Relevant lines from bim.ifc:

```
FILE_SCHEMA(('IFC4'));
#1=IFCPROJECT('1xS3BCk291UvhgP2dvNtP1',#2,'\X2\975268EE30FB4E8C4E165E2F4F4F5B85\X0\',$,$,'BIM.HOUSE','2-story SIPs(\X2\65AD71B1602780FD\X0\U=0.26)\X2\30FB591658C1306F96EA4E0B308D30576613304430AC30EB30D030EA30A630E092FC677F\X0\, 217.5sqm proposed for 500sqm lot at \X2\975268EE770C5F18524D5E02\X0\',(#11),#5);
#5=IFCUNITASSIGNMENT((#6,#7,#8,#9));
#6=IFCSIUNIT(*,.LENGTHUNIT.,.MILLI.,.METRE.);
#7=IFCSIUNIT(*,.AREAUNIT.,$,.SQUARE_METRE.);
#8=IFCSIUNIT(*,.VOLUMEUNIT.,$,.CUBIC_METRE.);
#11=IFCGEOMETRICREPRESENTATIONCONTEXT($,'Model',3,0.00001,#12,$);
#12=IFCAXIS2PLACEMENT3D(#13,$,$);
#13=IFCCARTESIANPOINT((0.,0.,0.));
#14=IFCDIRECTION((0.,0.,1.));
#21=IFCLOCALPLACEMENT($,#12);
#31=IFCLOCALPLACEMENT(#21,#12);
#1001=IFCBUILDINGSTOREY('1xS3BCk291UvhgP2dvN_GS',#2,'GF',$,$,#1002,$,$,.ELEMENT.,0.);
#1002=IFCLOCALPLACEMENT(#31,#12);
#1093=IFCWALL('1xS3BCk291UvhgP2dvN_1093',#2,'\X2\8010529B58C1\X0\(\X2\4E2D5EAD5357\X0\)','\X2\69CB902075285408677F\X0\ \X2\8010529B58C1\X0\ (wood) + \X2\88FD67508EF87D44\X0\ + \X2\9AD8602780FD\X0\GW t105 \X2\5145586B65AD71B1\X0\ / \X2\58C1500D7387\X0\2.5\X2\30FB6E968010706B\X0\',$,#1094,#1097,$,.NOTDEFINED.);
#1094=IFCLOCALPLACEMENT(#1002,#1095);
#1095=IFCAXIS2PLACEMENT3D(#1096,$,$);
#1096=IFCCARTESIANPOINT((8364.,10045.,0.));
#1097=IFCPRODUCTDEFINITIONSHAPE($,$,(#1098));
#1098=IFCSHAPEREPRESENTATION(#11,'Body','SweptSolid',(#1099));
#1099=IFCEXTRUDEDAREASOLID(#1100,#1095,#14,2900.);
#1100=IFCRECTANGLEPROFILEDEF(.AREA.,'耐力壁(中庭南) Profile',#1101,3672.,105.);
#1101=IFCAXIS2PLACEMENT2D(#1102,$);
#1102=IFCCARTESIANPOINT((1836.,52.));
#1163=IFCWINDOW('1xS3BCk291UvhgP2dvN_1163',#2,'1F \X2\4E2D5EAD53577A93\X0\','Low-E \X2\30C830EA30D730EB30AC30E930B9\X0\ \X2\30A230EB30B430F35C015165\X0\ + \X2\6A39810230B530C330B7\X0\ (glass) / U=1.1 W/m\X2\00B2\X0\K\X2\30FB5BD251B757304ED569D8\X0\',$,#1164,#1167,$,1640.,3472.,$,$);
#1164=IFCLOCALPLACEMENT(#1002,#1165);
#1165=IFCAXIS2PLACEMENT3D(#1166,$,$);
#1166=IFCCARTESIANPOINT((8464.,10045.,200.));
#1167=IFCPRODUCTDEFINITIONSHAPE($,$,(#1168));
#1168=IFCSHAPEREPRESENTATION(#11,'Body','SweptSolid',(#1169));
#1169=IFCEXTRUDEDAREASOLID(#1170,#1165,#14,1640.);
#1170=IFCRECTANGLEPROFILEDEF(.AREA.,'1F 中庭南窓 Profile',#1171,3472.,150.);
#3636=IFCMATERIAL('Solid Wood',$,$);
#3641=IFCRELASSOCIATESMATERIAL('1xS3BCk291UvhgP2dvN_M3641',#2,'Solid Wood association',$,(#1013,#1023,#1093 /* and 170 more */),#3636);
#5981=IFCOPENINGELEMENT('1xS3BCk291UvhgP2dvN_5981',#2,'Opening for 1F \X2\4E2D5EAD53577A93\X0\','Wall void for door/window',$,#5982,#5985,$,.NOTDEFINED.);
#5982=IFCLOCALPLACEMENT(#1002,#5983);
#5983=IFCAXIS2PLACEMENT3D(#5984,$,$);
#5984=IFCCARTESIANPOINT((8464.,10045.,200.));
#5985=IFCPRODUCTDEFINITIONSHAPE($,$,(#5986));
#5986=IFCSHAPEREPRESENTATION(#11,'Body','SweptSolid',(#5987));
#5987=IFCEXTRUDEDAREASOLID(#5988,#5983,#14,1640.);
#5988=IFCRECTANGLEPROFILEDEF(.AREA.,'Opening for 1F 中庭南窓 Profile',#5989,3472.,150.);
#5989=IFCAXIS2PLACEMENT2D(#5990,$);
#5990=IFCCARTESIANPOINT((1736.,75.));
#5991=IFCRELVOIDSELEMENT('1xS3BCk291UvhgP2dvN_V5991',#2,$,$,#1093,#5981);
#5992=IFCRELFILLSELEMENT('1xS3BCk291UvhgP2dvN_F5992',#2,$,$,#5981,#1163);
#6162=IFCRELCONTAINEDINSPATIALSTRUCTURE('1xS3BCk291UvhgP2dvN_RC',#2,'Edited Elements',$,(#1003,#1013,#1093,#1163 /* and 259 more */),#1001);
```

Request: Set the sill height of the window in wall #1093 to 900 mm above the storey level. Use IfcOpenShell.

```python
import numpy as np
import ifcopenshell
import ifcopenshell.api.geometry
import ifcopenshell.geom
import ifcopenshell.util.element
import ifcopenshell.util.placement
import ifcopenshell.util.shape
import ifcopenshell.util.unit

model = ifcopenshell.open("bim.ifc")
unit_scale = ifcopenshell.util.unit.calculate_unit_scale(model)

window = model.by_id(1163)
opening = window.FillsVoids[0].RelatingOpeningElement
storey = ifcopenshell.util.element.get_container(window, ifc_class="IfcBuildingStorey")
level = ifcopenshell.util.placement.get_local_placement(storey.ObjectPlacement)[2, 3]

# The opening's origin need not be at the sill, so measure its lowest point.
shape = ifcopenshell.geom.create_shape(ifcopenshell.geom.settings(), opening)
bottom = ifcopenshell.util.shape.get_shape_bottom_elevation(shape, shape.geometry) / unit_scale
dz = level + 900.0 - bottom

shift = np.array([0.0, 0.0, dz])
# The window is not placed relative to its opening, so move both.
for product in (opening, window):
    matrix = ifcopenshell.util.placement.get_local_placement(product.ObjectPlacement)
    matrix[:3, 3] += shift
    ifcopenshell.api.geometry.edit_object_placement(model, product=product, matrix=matrix, is_si=False)

print(f"moved by {dz * unit_scale:+.3f} m")

model.write("bim_updated.ifc")
```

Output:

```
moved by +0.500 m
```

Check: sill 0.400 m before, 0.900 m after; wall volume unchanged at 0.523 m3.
